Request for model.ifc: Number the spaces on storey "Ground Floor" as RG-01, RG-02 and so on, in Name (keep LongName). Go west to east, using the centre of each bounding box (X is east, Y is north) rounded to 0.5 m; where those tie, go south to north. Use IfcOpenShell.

First a look at what the model holds.

```python
import ifcopenshell
import ifcopenshell.util.element
import ifcopenshell.util.placement

model = ifcopenshell.open("model.ifc")
print(model.schema)
storey = next(s for s in model.by_type("IfcBuildingStorey") if s.Name == "Ground Floor")
spaces = [e for e in ifcopenshell.util.element.get_decomposition(storey) if e.is_a("IfcSpace")]
for e in sorted(spaces, key=lambda e: e.id()):
    origin = ifcopenshell.util.placement.get_local_placement(e.ObjectPlacement)[:3, 3]
    print(e.id(), e.Name, e.LongName, origin.round(2) + 0.0, sep=" | ")
```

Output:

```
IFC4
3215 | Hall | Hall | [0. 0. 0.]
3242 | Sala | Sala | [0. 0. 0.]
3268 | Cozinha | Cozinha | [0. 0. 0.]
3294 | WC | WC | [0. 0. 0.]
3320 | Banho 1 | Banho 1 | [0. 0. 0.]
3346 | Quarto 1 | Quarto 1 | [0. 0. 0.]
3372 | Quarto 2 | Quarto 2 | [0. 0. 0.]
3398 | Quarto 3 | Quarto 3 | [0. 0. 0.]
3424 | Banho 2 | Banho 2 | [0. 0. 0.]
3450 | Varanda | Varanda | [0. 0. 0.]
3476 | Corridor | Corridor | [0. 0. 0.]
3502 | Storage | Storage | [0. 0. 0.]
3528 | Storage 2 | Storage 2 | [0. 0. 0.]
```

```python
import ifcopenshell
import ifcopenshell.geom
import ifcopenshell.util.element
import ifcopenshell.util.shape

model = ifcopenshell.open("model.ifc")
settings = ifcopenshell.geom.settings()
settings.set("use-world-coords", True)


def centre(element):
    shape = ifcopenshell.geom.create_shape(settings, element)
    return ifcopenshell.util.shape.get_bbox_centroid(shape.geometry)


storey = next(s for s in model.by_type("IfcBuildingStorey") if s.Name == "Ground Floor")
spaces = [e for e in ifcopenshell.util.element.get_decomposition(storey) if e.is_a("IfcSpace")]

# Insertion points can sit at a corner or the storey origin, so sort by the geometry (in metres).
centres = {e: centre(e) for e in spaces}
spaces.sort(key=lambda e: (round(centres[e][0] / 0.5), centres[e][1]))

for i, e in enumerate(spaces, start=1):
    number = f"RG-{i:02d}"
    e.Name = number
    print(e.id(), number)

model.write("model_rev.ifc")
```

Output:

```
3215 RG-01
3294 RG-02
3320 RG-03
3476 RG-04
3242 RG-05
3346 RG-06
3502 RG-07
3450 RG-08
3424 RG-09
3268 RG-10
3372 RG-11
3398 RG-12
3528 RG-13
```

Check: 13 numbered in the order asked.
